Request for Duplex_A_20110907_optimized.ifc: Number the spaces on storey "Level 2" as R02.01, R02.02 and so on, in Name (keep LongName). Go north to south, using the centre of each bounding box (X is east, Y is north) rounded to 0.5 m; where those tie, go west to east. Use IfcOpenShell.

First a look at what the model holds.

```python
import ifcopenshell
import ifcopenshell.util.element
import ifcopenshell.util.placement

model = ifcopenshell.open("Duplex_A_20110907_optimized.ifc")
print(model.schema)
storey = next(s for s in model.by_type("IfcBuildingStorey") if s.Name == "Level 2")
spaces = [e for e in ifcopenshell.util.element.get_decomposition(storey) if e.is_a("IfcSpace")]
for e in sorted(spaces, key=lambda e: e.id()):
    origin = ifcopenshell.util.placement.get_local_placement(e.ObjectPlacement)[:3, 3]
    print(e.id(), e.Name, e.LongName, origin.round(2) + 0.0, sep=" | ")
```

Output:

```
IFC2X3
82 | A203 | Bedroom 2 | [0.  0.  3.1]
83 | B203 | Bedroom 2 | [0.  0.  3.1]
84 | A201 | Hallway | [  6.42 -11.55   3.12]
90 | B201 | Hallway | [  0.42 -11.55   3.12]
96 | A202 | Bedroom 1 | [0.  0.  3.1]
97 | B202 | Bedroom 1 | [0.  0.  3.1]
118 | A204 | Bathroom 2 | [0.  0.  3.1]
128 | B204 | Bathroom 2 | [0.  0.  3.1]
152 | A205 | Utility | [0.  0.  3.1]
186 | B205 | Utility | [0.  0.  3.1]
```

```python
import ifcopenshell
import ifcopenshell.geom
import ifcopenshell.util.element
import ifcopenshell.util.shape

model = ifcopenshell.open("Duplex_A_20110907_optimized.ifc")
settings = ifcopenshell.geom.settings()
settings.set("use-world-coords", True)


def centre(element):
    shape = ifcopenshell.geom.create_shape(settings, element)
    return ifcopenshell.util.shape.get_bbox_centroid(shape.geometry)


storey = next(s for s in model.by_type("IfcBuildingStorey") if s.Name == "Level 2")
spaces = [e for e in ifcopenshell.util.element.get_decomposition(storey) if e.is_a("IfcSpace")]

# Insertion points can sit at a corner or the storey origin, so sort by the geometry (in metres).
centres = {e: centre(e) for e in spaces}
spaces.sort(key=lambda e: (-round(centres[e][1] / 0.5), centres[e][0]))

for i, e in enumerate(spaces, start=1):
    number = f"R02.{i:02d}"
    e.Name = number
    print(e.id(), number)

model.write("Duplex_A_20110907_optimized_updated.ifc")
```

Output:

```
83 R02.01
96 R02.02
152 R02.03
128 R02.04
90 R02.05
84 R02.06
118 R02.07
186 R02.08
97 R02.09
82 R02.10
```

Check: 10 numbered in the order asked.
